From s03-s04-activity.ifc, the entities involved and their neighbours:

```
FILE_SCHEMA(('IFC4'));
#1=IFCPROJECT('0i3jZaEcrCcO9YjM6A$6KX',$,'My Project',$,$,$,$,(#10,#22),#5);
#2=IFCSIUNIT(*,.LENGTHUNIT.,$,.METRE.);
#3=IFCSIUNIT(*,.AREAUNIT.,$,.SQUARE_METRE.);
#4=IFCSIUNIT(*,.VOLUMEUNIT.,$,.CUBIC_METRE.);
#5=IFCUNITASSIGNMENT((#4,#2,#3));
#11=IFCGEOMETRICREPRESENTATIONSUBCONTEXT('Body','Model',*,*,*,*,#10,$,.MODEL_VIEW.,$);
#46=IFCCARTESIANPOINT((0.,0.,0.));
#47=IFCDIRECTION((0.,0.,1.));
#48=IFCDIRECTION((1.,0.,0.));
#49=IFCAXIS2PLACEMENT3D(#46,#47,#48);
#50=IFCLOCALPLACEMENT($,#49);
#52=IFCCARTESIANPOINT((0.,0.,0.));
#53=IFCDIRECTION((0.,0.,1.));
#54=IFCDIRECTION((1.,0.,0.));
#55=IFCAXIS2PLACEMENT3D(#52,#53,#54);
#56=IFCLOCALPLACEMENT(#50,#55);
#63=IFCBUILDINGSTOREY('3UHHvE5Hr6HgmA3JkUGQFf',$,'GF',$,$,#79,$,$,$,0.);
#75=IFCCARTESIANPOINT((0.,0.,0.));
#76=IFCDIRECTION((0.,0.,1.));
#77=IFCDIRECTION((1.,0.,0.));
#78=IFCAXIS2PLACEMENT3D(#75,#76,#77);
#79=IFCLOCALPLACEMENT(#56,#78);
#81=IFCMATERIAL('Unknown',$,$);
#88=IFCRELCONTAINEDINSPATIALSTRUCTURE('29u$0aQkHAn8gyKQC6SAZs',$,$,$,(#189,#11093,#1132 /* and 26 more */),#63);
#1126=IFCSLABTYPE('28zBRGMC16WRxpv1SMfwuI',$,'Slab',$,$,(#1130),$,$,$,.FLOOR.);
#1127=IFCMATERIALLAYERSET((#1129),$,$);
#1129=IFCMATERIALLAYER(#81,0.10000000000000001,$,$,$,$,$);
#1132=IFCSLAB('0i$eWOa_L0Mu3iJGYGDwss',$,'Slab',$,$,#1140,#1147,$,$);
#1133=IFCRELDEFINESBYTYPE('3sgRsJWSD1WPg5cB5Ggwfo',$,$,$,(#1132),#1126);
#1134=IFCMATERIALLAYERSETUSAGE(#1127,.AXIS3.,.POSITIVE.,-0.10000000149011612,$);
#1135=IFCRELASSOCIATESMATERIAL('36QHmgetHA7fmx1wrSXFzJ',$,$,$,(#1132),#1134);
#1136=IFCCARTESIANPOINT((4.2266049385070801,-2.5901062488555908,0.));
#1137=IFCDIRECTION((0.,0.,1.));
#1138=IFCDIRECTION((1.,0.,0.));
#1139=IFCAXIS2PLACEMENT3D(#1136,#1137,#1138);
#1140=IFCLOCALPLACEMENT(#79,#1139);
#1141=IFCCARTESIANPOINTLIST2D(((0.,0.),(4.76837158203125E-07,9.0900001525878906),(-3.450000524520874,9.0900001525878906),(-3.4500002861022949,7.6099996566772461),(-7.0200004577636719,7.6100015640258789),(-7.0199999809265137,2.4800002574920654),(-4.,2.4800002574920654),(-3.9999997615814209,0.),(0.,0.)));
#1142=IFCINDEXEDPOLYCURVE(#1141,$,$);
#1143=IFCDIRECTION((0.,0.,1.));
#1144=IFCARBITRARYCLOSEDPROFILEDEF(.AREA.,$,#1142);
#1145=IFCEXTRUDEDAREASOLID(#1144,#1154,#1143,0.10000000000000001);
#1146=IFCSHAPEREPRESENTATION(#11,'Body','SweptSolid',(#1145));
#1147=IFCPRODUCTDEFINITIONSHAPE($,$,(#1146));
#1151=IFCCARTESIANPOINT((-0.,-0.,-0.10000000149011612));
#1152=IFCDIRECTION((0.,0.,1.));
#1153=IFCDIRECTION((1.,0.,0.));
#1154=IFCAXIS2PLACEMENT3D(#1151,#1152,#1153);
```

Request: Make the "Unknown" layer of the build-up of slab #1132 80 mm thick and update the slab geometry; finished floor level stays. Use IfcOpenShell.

```python
import ifcopenshell
import ifcopenshell.util.element
import ifcopenshell.util.representation
import ifcopenshell.util.unit

model = ifcopenshell.open("s03-s04-activity.ifc")
unit_scale = ifcopenshell.util.unit.calculate_unit_scale(model)

layer_set = model.by_id(1127)
layer = next(l for l in layer_set.MaterialLayers if l.Material and l.Material.Name == "Unknown")
change = 0.08 / unit_scale - layer.LayerThickness
layer.LayerThickness += change

# Geometry does not follow the layer set by itself.
slabs = [e for e in ifcopenshell.util.element.get_elements_by_material(model, layer_set) if e.is_a("IfcSlab")]
for slab in sorted(slabs, key=lambda e: e.id()):
    body = ifcopenshell.util.representation.get_representation(slab, "Model", "Body")
    solid = body.Items[0]
    old_depth = solid.Depth
    solid.Depth += change
    # Extruded upwards: lower the start of the extrusion so the top stays.
    x, y, z = solid.Position.Location.Coordinates
    solid.Position.Location = model.createIfcCartesianPoint((x, y, z - change))
    print(slab.id(), f"{old_depth:g} -> {solid.Depth:g}")

# The layers are counted up from the underside, which has moved.
for usage in {ifcopenshell.util.element.get_material(slab) for slab in slabs}:
    usage.OffsetFromReferenceLine -= change

model.write("s03-s04-activity_updated.ifc")
```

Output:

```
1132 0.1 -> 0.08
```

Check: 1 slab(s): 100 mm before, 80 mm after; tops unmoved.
